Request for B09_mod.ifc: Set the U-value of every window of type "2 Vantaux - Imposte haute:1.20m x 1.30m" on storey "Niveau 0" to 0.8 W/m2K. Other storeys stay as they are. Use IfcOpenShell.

First a look at what the model holds.

```python
import ifcopenshell
import ifcopenshell.util.element

model = ifcopenshell.open("B09_mod.ifc")
print(model.schema)
storey = next(s for s in model.by_type("IfcBuildingStorey") if s.Name == "Niveau 0")
windows = [e for e in ifcopenshell.util.element.get_decomposition(storey) if e.is_a("IfcWindow")]
seen = {}
for e in windows:
    element_type = ifcopenshell.util.element.get_type(e)
    key = (element_type.Name if element_type != e and element_type else None, ifcopenshell.util.element.get_pset(e, "Pset_WindowCommon", "ThermalTransmittance"))
    seen[key] = seen.get(key, 0) + 1
for (name, value), count in sorted(seen.items(), key=str):
    print(count, "x", name, "|", value)
```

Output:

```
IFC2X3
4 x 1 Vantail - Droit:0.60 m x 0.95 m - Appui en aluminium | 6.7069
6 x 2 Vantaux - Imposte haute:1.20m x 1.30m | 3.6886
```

```python
import ifcopenshell
import ifcopenshell.api.pset
import ifcopenshell.util.element

model = ifcopenshell.open("B09_mod.ifc")

storey = next(s for s in model.by_type("IfcBuildingStorey") if s.Name == "Niveau 0")
windows = [e for e in ifcopenshell.util.element.get_decomposition(storey) if e.is_a("IfcWindow")]

count = 0
for e in windows:
    element_type = ifcopenshell.util.element.get_type(e)
    if element_type in (None, e) or element_type.Name != "2 Vantaux - Imposte haute:1.20m x 1.30m":
        continue
    # add_pset returns the element's existing set when there is one.
    pset = ifcopenshell.api.pset.add_pset(model, product=e, name="Pset_WindowCommon")
    ifcopenshell.api.pset.edit_pset(model, pset=pset, properties={"ThermalTransmittance": 0.8})
    count += 1

print(count, "windows updated")

model.write("B09_mod_updated.ifc")
```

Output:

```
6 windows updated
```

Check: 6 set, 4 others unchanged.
